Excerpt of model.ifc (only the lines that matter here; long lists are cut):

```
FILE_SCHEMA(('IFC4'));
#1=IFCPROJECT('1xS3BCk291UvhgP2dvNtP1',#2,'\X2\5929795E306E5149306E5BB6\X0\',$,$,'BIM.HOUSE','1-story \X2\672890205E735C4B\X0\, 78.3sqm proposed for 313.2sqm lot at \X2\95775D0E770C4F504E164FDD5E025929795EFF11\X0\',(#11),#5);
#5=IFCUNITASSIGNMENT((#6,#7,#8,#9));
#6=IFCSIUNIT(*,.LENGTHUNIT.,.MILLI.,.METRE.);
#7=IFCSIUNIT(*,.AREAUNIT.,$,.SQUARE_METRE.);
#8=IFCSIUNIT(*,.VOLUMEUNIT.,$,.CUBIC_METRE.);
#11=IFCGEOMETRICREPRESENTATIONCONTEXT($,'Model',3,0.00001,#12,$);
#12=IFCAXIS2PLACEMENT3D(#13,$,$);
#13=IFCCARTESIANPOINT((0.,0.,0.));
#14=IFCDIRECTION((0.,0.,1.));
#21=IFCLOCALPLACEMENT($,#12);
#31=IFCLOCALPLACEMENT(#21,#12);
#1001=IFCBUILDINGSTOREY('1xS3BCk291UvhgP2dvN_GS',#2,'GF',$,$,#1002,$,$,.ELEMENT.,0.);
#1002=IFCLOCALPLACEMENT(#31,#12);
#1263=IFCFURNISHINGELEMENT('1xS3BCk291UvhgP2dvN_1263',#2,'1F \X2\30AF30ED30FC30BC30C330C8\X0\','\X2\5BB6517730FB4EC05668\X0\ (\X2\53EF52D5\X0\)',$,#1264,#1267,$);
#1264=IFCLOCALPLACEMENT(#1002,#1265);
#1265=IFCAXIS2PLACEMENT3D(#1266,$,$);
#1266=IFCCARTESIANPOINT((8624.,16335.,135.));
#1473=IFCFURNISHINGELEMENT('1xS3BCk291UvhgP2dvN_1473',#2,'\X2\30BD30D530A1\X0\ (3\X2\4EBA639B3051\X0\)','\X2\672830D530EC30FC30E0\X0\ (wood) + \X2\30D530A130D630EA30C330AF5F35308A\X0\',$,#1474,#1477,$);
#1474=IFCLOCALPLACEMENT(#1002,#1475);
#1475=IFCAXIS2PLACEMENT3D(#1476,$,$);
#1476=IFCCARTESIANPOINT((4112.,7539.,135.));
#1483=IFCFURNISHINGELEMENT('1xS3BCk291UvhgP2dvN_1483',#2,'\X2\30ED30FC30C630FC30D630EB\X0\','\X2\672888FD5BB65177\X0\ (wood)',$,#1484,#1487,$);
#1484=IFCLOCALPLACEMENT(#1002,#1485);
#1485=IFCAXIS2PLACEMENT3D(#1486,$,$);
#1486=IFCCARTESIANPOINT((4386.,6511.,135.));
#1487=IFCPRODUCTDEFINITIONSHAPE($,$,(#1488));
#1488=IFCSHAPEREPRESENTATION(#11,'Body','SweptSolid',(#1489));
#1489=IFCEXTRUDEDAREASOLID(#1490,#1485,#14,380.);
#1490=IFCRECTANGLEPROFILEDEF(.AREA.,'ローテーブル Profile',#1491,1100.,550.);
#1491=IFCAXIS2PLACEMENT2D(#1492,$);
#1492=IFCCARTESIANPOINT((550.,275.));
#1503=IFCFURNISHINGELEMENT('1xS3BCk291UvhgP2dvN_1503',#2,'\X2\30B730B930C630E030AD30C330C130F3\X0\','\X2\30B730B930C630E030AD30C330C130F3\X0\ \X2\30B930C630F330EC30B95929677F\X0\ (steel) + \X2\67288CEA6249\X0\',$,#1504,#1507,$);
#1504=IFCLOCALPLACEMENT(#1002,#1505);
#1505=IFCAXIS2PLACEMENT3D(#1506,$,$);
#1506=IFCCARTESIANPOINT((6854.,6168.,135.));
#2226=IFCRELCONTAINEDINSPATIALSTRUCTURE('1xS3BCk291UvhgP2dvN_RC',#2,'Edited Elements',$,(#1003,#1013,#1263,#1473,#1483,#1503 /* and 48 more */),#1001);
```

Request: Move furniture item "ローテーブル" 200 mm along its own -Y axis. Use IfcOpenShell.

```python
import ifcopenshell
import ifcopenshell.api.geometry
import ifcopenshell.util.placement
import ifcopenshell.util.unit

model = ifcopenshell.open("model.ifc")
unit_scale = ifcopenshell.util.unit.calculate_unit_scale(model)

item = model.by_guid("1xS3BCk291UvhgP2dvN_1483")
matrix = ifcopenshell.util.placement.get_local_placement(item.ObjectPlacement)
matrix[:3, 3] -= matrix[:3, 1] * 0.2 / unit_scale
ifcopenshell.api.geometry.edit_object_placement(model, product=item, matrix=matrix, is_si=False)

print(ifcopenshell.util.placement.get_local_placement(item.ObjectPlacement).round(3) + 0.0)

model.write("model-out.ifc")
```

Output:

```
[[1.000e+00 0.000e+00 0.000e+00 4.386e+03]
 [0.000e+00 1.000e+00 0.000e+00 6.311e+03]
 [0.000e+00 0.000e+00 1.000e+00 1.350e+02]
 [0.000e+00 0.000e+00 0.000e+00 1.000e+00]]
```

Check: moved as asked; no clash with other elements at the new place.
